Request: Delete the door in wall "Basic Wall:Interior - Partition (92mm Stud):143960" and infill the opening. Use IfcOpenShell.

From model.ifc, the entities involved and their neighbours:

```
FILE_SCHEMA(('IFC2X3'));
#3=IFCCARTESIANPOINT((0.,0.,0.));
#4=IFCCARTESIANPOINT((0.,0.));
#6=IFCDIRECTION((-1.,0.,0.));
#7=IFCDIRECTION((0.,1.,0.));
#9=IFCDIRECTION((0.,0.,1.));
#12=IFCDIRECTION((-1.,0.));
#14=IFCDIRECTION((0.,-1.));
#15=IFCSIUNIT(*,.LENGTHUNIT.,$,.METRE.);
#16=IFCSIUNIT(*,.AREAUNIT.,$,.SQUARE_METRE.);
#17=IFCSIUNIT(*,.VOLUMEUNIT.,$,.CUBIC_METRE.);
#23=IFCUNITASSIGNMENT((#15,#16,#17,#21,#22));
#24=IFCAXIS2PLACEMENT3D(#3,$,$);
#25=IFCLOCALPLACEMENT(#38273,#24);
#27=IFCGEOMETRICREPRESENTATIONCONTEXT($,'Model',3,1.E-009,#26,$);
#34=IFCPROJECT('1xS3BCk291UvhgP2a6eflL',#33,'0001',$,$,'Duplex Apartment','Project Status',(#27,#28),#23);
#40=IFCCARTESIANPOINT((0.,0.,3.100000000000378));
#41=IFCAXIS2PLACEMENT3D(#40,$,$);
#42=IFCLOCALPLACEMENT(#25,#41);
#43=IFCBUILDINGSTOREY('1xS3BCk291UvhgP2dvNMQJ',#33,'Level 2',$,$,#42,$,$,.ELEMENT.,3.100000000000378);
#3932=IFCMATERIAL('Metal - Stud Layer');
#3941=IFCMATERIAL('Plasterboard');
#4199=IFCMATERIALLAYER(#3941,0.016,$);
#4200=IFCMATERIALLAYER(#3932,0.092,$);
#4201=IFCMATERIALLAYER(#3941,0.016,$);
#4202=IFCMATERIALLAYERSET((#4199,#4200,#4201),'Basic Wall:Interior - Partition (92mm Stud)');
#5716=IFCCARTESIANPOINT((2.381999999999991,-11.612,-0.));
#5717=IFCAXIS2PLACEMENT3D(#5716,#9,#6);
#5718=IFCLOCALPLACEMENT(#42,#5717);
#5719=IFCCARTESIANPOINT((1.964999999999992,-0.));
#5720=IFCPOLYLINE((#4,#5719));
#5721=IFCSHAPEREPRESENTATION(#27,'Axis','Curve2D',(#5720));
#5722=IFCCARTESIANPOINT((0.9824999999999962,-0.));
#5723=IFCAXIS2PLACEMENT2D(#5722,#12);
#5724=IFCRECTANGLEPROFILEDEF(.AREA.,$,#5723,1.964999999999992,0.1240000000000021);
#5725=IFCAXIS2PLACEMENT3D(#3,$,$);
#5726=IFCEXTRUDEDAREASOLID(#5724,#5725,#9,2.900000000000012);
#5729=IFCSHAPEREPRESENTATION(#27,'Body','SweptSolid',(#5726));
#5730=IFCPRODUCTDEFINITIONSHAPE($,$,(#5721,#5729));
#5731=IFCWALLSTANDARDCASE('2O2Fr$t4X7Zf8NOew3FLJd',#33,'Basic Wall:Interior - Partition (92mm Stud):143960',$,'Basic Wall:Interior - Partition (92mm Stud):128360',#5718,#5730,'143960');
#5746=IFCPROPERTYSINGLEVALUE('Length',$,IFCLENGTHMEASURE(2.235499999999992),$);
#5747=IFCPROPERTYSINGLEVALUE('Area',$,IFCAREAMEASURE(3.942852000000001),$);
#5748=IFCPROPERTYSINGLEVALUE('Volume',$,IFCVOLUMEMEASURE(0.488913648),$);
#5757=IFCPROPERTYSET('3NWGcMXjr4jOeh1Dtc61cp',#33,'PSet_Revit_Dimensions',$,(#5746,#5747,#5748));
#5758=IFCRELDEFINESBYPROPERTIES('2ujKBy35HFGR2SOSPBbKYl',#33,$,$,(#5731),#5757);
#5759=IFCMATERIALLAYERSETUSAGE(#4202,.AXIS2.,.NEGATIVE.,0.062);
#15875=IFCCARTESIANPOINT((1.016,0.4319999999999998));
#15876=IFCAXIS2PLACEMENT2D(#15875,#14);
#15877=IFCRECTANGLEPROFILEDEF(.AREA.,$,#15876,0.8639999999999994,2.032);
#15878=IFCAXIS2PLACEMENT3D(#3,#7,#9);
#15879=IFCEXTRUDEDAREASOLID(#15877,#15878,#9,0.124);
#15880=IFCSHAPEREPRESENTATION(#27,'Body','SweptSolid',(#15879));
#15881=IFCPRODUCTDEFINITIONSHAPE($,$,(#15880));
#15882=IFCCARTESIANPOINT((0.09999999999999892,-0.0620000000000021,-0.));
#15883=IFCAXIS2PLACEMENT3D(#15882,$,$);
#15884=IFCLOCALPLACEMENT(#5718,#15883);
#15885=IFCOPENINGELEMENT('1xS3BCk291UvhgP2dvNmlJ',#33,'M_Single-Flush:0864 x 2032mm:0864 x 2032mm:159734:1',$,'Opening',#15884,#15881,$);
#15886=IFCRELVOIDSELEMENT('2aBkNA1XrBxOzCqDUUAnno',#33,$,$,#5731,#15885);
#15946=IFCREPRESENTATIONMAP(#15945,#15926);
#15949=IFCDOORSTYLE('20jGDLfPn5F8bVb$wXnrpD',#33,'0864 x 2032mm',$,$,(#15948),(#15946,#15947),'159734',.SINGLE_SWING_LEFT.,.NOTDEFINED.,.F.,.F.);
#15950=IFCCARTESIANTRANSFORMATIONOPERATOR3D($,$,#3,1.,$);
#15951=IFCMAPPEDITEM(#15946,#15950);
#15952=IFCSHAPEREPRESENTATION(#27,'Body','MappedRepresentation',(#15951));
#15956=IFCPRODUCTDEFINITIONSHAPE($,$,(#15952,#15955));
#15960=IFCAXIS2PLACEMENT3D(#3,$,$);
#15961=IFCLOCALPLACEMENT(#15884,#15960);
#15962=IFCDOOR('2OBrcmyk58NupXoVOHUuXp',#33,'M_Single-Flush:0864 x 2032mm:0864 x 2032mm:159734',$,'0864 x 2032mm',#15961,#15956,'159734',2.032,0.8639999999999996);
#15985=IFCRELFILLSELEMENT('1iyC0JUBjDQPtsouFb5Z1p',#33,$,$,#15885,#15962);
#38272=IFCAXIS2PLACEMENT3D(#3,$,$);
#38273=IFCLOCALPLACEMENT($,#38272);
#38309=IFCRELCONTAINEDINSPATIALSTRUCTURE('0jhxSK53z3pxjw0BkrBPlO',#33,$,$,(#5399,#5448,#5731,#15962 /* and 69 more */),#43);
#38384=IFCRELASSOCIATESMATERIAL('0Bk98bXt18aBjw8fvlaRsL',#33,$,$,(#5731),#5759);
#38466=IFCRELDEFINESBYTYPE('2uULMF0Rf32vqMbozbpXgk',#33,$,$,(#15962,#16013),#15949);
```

```python
import ifcopenshell
import ifcopenshell.api.feature
import ifcopenshell.api.pset
import ifcopenshell.api.root
import ifcopenshell.geom
import ifcopenshell.util.element
import ifcopenshell.util.shape
import ifcopenshell.util.unit

model = ifcopenshell.open("model.ifc")
area_scale = ifcopenshell.util.unit.calculate_unit_scale(model, "AREAUNIT")
volume_scale = ifcopenshell.util.unit.calculate_unit_scale(model, "VOLUMEUNIT")
settings = ifcopenshell.geom.settings()


def volume(element):
    """Net volume in cubic metres, openings subtracted."""
    shape = ifcopenshell.geom.create_shape(settings, element)
    return ifcopenshell.util.shape.get_volume(shape.geometry)


door = model.by_guid("2OBrcmyk58NupXoVOHUuXp")
opening = door.FillsVoids[0].RelatingOpeningElement
wall = opening.VoidsElements[0].RelatingBuildingElement
before = volume(wall)

ifcopenshell.api.root.remove_product(model, product=door)
ifcopenshell.api.feature.remove_feature(model, feature=opening)

after = volume(wall)
thickness = 0.124  # wall thickness in metres

# Update the wall's stored quantities.
pset = model.by_id(ifcopenshell.util.element.get_pset(wall, "PSet_Revit_Dimensions", should_inherit=False)["id"])
ifcopenshell.api.pset.edit_pset(model, pset=pset, properties={
    "Area": model.create_entity("IfcAreaMeasure", after / thickness / area_scale),
    "Volume": model.create_entity("IfcVolumeMeasure", after / volume_scale),
})

print(f"wall volume {before:.3f} -> {after:.3f} m3")

model.write("model_v2.ifc")
```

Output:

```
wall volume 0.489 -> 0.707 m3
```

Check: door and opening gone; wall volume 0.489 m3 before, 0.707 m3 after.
